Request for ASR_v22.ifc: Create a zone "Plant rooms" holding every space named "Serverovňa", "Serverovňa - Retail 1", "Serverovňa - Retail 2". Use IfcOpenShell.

First a look at what the model holds.

```python
import ifcopenshell

model = ifcopenshell.open("ASR_v22.ifc")
print(model.schema)
seen = {}
for space in model.by_type("IfcSpace"):
    seen[space.LongName] = seen.get(space.LongName, 0) + 1
for name, count in sorted(seen.items(), key=str):
    print(count, "x", name)
print("zones:", [z.Name for z in model.by_type("IfcZone")][:20])
```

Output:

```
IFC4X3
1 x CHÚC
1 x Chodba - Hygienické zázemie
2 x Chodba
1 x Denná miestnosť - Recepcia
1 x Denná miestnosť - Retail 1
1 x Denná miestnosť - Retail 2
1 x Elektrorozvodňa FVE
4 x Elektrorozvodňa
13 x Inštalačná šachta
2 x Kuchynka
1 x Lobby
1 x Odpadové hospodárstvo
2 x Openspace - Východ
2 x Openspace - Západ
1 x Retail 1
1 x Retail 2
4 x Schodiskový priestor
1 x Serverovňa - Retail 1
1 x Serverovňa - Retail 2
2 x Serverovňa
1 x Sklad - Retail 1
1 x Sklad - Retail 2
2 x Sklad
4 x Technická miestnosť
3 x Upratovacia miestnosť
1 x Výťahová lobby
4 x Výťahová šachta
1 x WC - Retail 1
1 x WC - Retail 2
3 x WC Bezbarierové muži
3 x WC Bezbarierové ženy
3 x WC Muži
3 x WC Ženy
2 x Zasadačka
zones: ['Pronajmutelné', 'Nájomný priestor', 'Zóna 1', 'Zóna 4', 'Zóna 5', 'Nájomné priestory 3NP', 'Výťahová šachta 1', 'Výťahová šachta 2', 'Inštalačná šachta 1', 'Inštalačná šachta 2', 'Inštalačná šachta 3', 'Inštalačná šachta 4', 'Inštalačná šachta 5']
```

```python
import ifcopenshell
import ifcopenshell.api.group
import ifcopenshell.api.root

model = ifcopenshell.open("ASR_v22.ifc")

names = {"Serverovňa", "Serverovňa - Retail 1", "Serverovňa - Retail 2"}
spaces = [s for s in model.by_type("IfcSpace") if s.LongName in names]

zone = ifcopenshell.api.root.create_entity(model, ifc_class="IfcZone", name="Plant rooms")
ifcopenshell.api.group.assign_group(model, products=spaces, group=zone)
print(len(spaces), "spaces in", zone.Name)

model.write("ASR_v22_edited.ifc")
```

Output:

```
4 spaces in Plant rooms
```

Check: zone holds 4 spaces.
